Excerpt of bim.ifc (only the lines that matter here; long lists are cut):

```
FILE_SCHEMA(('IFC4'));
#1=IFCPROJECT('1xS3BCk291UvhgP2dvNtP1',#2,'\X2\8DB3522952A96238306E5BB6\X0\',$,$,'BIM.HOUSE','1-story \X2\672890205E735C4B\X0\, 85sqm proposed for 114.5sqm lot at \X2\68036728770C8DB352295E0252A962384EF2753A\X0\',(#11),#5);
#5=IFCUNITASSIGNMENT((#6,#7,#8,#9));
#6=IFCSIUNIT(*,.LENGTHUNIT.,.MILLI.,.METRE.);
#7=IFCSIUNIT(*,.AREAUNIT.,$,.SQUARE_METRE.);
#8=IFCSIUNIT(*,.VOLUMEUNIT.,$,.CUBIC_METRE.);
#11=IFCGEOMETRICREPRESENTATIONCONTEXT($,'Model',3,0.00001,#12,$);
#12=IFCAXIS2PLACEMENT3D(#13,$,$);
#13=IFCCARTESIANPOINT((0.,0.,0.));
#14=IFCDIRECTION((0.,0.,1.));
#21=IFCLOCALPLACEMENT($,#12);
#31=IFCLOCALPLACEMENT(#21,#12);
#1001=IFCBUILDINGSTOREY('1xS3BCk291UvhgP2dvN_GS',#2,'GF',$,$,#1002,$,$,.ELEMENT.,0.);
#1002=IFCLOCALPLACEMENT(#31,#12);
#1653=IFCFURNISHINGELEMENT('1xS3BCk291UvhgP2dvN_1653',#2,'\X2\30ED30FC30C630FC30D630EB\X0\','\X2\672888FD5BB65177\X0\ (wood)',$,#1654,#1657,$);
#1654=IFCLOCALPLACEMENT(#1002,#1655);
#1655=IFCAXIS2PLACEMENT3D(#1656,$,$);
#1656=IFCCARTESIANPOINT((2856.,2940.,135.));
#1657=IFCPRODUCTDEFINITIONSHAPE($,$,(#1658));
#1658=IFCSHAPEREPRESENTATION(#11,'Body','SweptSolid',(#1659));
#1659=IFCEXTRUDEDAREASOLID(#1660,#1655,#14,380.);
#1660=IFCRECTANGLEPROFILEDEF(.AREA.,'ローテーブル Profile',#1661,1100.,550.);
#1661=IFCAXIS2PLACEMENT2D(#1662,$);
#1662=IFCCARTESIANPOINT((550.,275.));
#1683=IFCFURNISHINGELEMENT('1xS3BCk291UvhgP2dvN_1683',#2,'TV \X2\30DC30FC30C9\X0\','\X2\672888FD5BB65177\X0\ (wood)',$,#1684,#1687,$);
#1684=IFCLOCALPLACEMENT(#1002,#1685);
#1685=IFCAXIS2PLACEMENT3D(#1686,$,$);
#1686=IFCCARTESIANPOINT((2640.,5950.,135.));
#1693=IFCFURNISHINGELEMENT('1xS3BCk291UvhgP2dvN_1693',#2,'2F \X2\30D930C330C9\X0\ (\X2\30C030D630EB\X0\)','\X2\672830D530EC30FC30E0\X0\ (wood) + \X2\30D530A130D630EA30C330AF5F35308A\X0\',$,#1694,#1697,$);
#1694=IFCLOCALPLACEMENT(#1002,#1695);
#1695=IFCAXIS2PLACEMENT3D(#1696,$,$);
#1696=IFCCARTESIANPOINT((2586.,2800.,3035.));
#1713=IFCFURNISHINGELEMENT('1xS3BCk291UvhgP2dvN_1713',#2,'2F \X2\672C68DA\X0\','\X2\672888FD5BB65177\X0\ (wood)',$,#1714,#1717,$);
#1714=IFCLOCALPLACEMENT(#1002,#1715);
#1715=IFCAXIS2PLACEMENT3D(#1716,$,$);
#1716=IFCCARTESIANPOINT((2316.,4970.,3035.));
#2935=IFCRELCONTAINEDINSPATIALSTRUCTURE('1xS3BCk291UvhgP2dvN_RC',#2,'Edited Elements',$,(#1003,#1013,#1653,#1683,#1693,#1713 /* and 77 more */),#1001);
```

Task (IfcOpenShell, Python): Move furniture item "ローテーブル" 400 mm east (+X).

```python
import ifcopenshell
import ifcopenshell.api.geometry
import ifcopenshell.util.placement
import ifcopenshell.util.unit

model = ifcopenshell.open("bim.ifc")
unit_scale = ifcopenshell.util.unit.calculate_unit_scale(model)

item = model.by_guid("1xS3BCk291UvhgP2dvN_1653")
matrix = ifcopenshell.util.placement.get_local_placement(item.ObjectPlacement)
matrix[0, 3] += 0.4 / unit_scale
ifcopenshell.api.geometry.edit_object_placement(model, product=item, matrix=matrix, is_si=False)

print(ifcopenshell.util.placement.get_local_placement(item.ObjectPlacement).round(3) + 0.0)

model.write("bim_v2.ifc")
```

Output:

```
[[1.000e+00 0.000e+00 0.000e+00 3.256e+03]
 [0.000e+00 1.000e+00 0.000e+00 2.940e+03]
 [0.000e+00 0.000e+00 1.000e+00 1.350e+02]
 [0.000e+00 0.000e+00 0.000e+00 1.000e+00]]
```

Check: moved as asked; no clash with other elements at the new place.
